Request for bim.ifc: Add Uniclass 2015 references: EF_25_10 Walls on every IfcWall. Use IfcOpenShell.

First a look at what the model holds.

```python
import ifcopenshell

model = ifcopenshell.open("bim.ifc")
print(model.schema)
print("classifications:", [c.Name for c in model.by_type("IfcClassification")])
for ifc_class in ("IfcDoor", "IfcRoof", "IfcStair", "IfcWall", "IfcWindow"):
    print(ifc_class, len(model.by_type(ifc_class)))
```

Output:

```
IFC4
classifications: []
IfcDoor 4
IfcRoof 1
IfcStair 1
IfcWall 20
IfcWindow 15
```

```python
import ifcopenshell
import ifcopenshell.api.classification

model = ifcopenshell.open("bim.ifc")

system = ifcopenshell.api.classification.add_classification(model, classification="Uniclass 2015")

codes = {
    "IfcWall": ("EF_25_10", "Walls"),
}
for ifc_class, (code, name) in codes.items():
    products = model.by_type(ifc_class)
    ifcopenshell.api.classification.add_reference(
        model, products=products, classification=system, identification=code, name=name
    )
    print(code, len(products))

model.write("bim_rev.ifc")
```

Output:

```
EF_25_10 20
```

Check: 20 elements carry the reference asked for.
